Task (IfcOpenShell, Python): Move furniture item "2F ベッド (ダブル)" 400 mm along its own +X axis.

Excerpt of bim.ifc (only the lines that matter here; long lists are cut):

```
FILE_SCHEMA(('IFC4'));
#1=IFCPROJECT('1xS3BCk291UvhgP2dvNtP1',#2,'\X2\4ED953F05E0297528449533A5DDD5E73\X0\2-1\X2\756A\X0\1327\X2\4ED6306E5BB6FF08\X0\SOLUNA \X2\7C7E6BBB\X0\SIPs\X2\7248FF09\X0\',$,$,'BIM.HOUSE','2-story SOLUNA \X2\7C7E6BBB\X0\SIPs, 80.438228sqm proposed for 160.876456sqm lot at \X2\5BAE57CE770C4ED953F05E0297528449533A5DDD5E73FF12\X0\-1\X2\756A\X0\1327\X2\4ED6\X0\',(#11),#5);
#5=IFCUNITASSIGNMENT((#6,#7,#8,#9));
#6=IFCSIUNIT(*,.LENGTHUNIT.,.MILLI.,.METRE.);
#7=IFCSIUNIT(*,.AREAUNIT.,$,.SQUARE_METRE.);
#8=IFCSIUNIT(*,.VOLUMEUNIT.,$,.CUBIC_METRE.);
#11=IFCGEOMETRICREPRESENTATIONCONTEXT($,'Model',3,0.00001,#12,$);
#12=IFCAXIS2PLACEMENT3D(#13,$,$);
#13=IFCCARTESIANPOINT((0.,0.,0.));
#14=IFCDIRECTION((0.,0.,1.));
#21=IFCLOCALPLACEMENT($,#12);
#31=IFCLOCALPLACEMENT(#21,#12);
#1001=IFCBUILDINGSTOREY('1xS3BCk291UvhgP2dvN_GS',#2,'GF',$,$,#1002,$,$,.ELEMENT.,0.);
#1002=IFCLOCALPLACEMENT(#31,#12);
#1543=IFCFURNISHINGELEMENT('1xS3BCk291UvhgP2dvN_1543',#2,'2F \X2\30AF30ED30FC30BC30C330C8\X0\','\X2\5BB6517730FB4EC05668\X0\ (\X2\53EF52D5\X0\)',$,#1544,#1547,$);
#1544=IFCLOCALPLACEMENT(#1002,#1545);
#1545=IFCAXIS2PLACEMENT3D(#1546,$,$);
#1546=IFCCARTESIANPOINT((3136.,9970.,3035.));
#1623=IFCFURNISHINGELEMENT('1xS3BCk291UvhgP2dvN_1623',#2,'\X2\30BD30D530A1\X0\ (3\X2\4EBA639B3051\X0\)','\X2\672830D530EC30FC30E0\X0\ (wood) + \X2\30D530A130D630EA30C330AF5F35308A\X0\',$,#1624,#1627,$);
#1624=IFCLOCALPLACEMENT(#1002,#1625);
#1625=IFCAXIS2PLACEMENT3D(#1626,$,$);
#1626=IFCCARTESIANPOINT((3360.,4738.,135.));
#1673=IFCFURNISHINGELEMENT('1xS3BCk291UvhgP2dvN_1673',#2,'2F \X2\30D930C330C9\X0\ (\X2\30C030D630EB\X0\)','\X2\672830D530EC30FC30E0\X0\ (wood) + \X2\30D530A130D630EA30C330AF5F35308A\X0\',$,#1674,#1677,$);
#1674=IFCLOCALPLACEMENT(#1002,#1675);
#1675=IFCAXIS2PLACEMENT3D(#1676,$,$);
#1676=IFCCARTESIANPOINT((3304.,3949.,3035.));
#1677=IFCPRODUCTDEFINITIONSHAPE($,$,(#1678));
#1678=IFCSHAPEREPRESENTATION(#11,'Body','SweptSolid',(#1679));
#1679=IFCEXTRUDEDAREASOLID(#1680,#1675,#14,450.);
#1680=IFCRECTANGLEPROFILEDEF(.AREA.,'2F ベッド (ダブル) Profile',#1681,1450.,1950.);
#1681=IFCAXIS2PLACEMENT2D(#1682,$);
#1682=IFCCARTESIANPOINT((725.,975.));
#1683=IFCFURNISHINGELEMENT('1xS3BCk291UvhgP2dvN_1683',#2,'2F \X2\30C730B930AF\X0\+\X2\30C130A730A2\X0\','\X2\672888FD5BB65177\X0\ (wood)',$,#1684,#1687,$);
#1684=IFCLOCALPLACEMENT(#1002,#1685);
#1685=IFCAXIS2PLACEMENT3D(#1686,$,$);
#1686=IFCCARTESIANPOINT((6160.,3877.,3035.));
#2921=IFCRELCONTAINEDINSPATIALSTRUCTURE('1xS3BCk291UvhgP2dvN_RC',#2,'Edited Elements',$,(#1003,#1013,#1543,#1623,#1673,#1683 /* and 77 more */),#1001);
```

```python
import ifcopenshell
import ifcopenshell.api.geometry
import ifcopenshell.util.placement
import ifcopenshell.util.unit

model = ifcopenshell.open("bim.ifc")
unit_scale = ifcopenshell.util.unit.calculate_unit_scale(model)

item = model.by_guid("1xS3BCk291UvhgP2dvN_1673")
matrix = ifcopenshell.util.placement.get_local_placement(item.ObjectPlacement)
matrix[:3, 3] += matrix[:3, 0] * 0.4 / unit_scale
ifcopenshell.api.geometry.edit_object_placement(model, product=item, matrix=matrix, is_si=False)

print(ifcopenshell.util.placement.get_local_placement(item.ObjectPlacement).round(3) + 0.0)

model.write("bim_updated.ifc")
```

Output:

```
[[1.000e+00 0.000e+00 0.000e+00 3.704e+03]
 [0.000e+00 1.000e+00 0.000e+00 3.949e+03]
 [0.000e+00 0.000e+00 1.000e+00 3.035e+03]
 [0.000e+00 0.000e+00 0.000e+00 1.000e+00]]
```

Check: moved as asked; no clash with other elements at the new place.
